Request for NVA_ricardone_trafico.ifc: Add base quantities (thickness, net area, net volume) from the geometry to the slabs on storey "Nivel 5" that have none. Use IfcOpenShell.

First a look at what the model holds.

```python
import ifcopenshell
import ifcopenshell.util.element
import ifcopenshell.util.unit

model = ifcopenshell.open("NVA_ricardone_trafico.ifc")
print(model.schema)
for unit_type in ("LENGTHUNIT", "AREAUNIT", "VOLUMEUNIT"):
    print(unit_type, ifcopenshell.util.unit.calculate_unit_scale(model, unit_type))
storey = next(s for s in model.by_type("IfcBuildingStorey") if s.Name == "Nivel 5")
slabs = [e for e in ifcopenshell.util.element.get_decomposition(storey) if e.is_a("IfcSlab")]
for e in sorted(slabs, key=lambda e: e.id()):
    print(e.id(), e.is_a(), e.Name, list(ifcopenshell.util.element.get_psets(e, qtos_only=True)), sep=" | ")
```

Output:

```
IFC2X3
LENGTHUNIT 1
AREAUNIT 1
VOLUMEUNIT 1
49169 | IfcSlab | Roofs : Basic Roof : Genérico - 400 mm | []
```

```python
import ifcopenshell
import ifcopenshell.api.pset
import ifcopenshell.geom
import ifcopenshell.util.element
import ifcopenshell.util.shape
import ifcopenshell.util.unit

model = ifcopenshell.open("NVA_ricardone_trafico.ifc")
unit_scale = ifcopenshell.util.unit.calculate_unit_scale(model)
area_scale = ifcopenshell.util.unit.calculate_unit_scale(model, "AREAUNIT")
volume_scale = ifcopenshell.util.unit.calculate_unit_scale(model, "VOLUMEUNIT")
settings = ifcopenshell.geom.settings()

storey = next(s for s in model.by_type("IfcBuildingStorey") if s.Name == "Nivel 5")
slabs = [e for e in ifcopenshell.util.element.get_decomposition(storey) if e.is_a("IfcSlab")]

for e in sorted(slabs, key=lambda e: e.id()):
    if ifcopenshell.util.element.get_psets(e, qtos_only=True, should_inherit=False):
        continue
    # Geometry comes back in metres, in the element's own axes.
    shape = ifcopenshell.geom.create_shape(settings, e)
    values = {
        "Width": ifcopenshell.util.shape.get_z(shape.geometry) / unit_scale,
        "NetArea": ifcopenshell.util.shape.get_footprint_area(shape.geometry) / area_scale,
        "NetVolume": ifcopenshell.util.shape.get_volume(shape.geometry) / volume_scale,
    }
    qto = ifcopenshell.api.pset.add_qto(model, product=e, name="BaseQuantities")
    ifcopenshell.api.pset.edit_qto(model, qto=qto, properties=values)
    print(e.id(), {k: round(v, 3) for k, v in values.items()})

model.write("NVA_ricardone_trafico_rev.ifc")
```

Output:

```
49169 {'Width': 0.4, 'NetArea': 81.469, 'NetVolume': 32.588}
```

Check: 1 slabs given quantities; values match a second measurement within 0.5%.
